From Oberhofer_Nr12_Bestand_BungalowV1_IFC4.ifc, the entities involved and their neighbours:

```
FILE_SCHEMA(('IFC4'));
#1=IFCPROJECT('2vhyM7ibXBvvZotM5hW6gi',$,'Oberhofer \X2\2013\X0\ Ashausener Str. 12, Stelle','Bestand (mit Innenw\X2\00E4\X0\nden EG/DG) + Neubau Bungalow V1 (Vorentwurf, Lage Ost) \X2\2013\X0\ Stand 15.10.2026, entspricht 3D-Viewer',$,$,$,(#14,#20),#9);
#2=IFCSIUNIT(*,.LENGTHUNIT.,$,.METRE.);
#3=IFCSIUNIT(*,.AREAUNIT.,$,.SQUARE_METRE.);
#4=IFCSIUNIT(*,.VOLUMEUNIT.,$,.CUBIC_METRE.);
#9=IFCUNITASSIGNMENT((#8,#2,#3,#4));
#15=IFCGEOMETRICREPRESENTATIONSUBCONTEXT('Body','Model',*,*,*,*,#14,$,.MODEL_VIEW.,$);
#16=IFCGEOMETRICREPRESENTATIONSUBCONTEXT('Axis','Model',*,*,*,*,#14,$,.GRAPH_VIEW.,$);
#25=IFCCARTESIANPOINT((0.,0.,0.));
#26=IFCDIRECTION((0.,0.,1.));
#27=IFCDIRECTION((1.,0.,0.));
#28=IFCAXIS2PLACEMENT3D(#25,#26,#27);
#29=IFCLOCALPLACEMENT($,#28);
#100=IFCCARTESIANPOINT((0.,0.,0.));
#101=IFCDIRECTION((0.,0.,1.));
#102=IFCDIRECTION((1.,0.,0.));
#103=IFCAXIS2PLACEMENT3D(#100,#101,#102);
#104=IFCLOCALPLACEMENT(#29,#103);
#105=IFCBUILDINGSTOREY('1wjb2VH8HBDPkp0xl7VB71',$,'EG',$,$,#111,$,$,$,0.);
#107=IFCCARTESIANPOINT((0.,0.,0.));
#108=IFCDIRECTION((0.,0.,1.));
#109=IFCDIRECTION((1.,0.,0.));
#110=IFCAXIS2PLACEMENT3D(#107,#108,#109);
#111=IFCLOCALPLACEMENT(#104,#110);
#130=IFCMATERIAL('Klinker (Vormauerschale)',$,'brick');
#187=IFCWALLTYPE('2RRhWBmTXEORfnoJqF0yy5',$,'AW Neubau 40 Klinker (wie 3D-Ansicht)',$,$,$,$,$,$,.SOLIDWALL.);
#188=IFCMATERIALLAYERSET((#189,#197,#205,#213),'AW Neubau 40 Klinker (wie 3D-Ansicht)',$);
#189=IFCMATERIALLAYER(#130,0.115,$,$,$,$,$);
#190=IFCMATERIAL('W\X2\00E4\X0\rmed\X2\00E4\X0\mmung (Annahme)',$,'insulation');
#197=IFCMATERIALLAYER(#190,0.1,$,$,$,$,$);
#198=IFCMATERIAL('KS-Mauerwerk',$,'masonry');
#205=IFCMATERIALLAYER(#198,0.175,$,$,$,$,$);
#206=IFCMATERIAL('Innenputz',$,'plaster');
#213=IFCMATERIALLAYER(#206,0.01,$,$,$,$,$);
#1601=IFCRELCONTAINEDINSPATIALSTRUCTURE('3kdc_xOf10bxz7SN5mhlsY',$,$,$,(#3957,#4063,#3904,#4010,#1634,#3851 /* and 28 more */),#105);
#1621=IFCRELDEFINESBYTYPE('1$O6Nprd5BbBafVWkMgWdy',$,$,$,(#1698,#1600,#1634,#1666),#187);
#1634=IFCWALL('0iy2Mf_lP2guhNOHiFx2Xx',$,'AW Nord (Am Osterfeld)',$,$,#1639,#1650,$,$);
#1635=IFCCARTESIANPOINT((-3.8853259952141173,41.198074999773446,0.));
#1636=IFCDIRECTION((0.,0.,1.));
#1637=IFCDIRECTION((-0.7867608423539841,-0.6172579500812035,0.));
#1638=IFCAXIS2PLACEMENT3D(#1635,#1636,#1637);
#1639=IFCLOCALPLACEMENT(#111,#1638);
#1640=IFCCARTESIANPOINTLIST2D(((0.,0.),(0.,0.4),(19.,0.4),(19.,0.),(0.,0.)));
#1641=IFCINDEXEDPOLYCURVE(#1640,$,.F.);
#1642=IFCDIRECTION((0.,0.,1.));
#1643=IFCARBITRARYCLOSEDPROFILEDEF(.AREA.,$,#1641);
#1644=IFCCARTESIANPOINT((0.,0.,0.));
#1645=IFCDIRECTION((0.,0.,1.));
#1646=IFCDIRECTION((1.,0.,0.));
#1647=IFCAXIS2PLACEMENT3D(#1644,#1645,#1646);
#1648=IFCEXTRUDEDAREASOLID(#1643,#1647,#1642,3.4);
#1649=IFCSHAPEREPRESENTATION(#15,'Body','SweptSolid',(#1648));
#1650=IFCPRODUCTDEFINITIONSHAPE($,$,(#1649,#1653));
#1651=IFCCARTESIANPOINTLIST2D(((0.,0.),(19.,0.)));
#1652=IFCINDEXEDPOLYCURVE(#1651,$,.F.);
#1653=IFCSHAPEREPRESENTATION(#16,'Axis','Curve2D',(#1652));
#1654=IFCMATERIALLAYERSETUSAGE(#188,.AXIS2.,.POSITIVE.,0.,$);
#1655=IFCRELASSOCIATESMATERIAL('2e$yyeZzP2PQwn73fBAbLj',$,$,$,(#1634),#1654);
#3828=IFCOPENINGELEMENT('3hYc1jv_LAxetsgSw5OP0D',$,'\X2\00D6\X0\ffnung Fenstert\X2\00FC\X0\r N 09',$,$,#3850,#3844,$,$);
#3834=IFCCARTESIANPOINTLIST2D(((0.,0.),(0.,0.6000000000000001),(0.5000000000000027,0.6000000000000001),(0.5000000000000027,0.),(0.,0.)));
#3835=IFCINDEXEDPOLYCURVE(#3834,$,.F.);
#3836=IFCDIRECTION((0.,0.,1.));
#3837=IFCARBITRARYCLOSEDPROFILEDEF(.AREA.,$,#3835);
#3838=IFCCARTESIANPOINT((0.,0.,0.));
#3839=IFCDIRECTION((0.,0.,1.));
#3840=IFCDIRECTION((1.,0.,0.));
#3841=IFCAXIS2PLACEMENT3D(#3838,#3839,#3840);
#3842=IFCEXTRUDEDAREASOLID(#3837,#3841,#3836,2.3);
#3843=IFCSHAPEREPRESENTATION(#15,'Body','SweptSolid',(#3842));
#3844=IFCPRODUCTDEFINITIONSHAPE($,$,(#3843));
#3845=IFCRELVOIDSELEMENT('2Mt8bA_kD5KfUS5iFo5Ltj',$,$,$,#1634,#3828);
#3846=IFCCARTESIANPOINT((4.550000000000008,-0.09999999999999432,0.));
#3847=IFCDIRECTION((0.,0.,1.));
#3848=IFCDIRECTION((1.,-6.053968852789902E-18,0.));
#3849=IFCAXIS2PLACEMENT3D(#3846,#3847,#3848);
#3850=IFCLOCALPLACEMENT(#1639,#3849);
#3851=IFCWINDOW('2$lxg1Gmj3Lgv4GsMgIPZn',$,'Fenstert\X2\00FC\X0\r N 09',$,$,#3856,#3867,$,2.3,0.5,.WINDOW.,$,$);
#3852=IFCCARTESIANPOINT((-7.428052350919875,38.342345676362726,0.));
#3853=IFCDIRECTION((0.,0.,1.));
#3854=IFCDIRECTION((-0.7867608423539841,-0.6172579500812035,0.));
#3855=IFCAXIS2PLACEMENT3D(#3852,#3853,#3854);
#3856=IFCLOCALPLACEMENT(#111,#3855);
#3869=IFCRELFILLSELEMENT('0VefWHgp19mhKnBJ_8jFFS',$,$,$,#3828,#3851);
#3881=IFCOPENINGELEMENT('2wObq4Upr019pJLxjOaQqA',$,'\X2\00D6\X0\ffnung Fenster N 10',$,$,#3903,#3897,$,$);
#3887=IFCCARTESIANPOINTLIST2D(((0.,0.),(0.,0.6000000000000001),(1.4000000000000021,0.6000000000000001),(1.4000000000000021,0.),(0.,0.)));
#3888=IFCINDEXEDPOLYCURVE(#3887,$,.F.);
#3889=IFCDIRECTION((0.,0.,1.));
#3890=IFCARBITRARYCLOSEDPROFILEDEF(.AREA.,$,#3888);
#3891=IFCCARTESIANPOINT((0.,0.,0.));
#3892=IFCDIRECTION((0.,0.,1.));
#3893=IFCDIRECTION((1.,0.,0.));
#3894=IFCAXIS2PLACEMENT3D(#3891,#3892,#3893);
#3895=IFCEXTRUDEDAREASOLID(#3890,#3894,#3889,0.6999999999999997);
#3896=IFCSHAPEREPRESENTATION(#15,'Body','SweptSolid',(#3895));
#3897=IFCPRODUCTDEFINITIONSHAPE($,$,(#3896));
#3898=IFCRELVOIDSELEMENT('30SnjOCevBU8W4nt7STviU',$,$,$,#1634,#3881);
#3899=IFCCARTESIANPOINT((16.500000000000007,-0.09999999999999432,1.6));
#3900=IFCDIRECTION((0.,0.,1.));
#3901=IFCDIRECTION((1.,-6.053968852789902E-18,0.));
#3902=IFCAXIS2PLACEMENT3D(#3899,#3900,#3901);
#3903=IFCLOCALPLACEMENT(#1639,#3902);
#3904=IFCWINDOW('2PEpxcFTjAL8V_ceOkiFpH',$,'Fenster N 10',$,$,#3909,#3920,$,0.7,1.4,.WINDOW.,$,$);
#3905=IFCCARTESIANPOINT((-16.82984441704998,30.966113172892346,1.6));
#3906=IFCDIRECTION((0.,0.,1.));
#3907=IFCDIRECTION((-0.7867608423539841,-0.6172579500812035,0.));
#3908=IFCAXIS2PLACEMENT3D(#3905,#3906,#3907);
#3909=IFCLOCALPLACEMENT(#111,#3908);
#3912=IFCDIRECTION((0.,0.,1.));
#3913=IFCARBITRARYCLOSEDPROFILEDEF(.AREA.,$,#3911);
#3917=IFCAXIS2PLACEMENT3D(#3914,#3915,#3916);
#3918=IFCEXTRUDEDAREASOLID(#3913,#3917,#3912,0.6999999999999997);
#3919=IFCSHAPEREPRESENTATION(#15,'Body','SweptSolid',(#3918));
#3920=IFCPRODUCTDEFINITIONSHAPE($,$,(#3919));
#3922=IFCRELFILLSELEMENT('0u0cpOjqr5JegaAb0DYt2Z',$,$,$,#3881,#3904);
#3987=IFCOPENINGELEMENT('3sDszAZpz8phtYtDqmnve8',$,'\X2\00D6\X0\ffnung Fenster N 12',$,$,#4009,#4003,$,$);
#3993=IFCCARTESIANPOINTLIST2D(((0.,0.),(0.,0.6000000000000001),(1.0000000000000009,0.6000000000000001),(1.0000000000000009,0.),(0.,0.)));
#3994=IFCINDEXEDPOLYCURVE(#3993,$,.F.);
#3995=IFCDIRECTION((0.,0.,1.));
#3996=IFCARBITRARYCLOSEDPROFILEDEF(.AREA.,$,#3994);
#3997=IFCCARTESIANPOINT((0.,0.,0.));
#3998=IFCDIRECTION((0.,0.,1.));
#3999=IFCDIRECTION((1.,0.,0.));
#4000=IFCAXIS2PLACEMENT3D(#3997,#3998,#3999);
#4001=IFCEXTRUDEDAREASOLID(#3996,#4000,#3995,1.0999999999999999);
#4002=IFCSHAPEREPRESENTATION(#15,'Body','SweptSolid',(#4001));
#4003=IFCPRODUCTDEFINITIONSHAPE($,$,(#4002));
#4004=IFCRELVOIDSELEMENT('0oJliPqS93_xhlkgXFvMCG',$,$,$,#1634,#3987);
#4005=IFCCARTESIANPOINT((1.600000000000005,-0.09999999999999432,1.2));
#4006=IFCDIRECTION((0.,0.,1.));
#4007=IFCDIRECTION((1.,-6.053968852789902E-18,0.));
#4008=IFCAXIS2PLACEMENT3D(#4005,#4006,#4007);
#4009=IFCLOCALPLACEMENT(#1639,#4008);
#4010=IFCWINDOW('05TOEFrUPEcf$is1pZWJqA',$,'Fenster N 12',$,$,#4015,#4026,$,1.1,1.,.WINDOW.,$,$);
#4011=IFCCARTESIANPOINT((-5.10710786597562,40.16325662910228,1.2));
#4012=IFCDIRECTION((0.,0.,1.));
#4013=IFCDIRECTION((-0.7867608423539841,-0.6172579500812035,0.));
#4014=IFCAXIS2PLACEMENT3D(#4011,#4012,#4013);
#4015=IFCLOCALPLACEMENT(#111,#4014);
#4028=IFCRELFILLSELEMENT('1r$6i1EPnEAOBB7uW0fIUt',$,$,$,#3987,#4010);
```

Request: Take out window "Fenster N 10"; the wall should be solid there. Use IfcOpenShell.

```python
import ifcopenshell
import ifcopenshell.api.feature
import ifcopenshell.api.root
import ifcopenshell.geom
import ifcopenshell.util.shape

model = ifcopenshell.open("Oberhofer_Nr12_Bestand_BungalowV1_IFC4.ifc")
settings = ifcopenshell.geom.settings()


def volume(element):
    """Net volume in cubic metres, openings subtracted."""
    shape = ifcopenshell.geom.create_shape(settings, element)
    return ifcopenshell.util.shape.get_volume(shape.geometry)


window = model.by_guid("2PEpxcFTjAL8V_ceOkiFpH")
opening = window.FillsVoids[0].RelatingOpeningElement
wall = opening.VoidsElements[0].RelatingBuildingElement
before = volume(wall)

ifcopenshell.api.root.remove_product(model, product=window)
ifcopenshell.api.feature.remove_feature(model, feature=opening)

after = volume(wall)

print(f"wall volume {before:.3f} -> {after:.3f} m3")

model.write("Oberhofer_Nr12_Bestand_BungalowV1_IFC4-out.ifc")
```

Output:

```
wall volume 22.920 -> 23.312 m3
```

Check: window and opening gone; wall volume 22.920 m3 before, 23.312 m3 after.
